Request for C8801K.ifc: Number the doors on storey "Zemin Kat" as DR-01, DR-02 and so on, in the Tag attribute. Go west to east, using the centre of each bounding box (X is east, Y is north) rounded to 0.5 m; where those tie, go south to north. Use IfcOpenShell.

First a look at what the model holds.

```python
import ifcopenshell
import ifcopenshell.util.element
import ifcopenshell.util.placement

model = ifcopenshell.open("C8801K.ifc")
print(model.schema)
storey = next(s for s in model.by_type("IfcBuildingStorey") if s.Name == "Zemin Kat")
doors = [e for e in ifcopenshell.util.element.get_decomposition(storey) if e.is_a("IfcDoor")]
for e in sorted(doors, key=lambda e: e.id()):
    origin = ifcopenshell.util.placement.get_local_placement(e.ObjectPlacement)[:3, 3]
    print(e.id(), e.Tag, e.Name, origin.round(2) + 0.0, sep=" | ")
```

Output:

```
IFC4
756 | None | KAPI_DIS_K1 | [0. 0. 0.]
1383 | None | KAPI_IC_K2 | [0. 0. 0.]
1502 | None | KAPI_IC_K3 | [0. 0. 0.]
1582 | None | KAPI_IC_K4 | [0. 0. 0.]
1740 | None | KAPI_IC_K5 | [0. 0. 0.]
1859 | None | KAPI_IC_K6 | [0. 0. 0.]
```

```python
import ifcopenshell
import ifcopenshell.geom
import ifcopenshell.util.element
import ifcopenshell.util.shape

model = ifcopenshell.open("C8801K.ifc")
settings = ifcopenshell.geom.settings()
settings.set("use-world-coords", True)


def centre(element):
    shape = ifcopenshell.geom.create_shape(settings, element)
    return ifcopenshell.util.shape.get_bbox_centroid(shape.geometry)


storey = next(s for s in model.by_type("IfcBuildingStorey") if s.Name == "Zemin Kat")
doors = [e for e in ifcopenshell.util.element.get_decomposition(storey) if e.is_a("IfcDoor")]

# Insertion points can sit at a corner or the storey origin, so sort by the geometry (in metres).
centres = {e: centre(e) for e in doors}
doors.sort(key=lambda e: (round(centres[e][0] / 0.5), centres[e][1]))

for i, e in enumerate(doors, start=1):
    number = f"DR-{i:02d}"
    e.Tag = number
    print(e.id(), number)

model.write("C8801K-out.ifc")
```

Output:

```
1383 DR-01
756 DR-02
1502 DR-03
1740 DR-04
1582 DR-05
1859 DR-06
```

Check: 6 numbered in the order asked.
